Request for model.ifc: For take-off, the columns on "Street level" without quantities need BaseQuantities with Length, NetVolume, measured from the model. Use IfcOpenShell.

First a look at what the model holds.

```python
import ifcopenshell
import ifcopenshell.util.element
import ifcopenshell.util.unit

model = ifcopenshell.open("model.ifc")
print(model.schema)
for unit_type in ("LENGTHUNIT", "AREAUNIT", "VOLUMEUNIT"):
    print(unit_type, ifcopenshell.util.unit.calculate_unit_scale(model, unit_type))
storey = next(s for s in model.by_type("IfcBuildingStorey") if s.Name == "Street level")
columns = [e for e in ifcopenshell.util.element.get_decomposition(storey) if e.is_a("IfcColumn")]
for e in sorted(columns, key=lambda e: e.id()):
    print(e.id(), e.is_a(), e.Name, list(ifcopenshell.util.element.get_psets(e, qtos_only=True)), sep=" | ")
```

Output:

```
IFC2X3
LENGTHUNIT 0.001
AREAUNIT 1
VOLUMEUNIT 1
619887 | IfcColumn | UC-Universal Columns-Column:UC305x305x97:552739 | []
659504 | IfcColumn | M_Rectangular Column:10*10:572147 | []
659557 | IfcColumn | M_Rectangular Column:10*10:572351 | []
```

```python
import ifcopenshell
import ifcopenshell.api.pset
import ifcopenshell.geom
import ifcopenshell.util.element
import ifcopenshell.util.shape
import ifcopenshell.util.unit

model = ifcopenshell.open("model.ifc")
unit_scale = ifcopenshell.util.unit.calculate_unit_scale(model)
volume_scale = ifcopenshell.util.unit.calculate_unit_scale(model, "VOLUMEUNIT")
settings = ifcopenshell.geom.settings()

storey = next(s for s in model.by_type("IfcBuildingStorey") if s.Name == "Street level")
columns = [e for e in ifcopenshell.util.element.get_decomposition(storey) if e.is_a("IfcColumn")]

for e in sorted(columns, key=lambda e: e.id()):
    if ifcopenshell.util.element.get_psets(e, qtos_only=True, should_inherit=False):
        continue
    # Geometry comes back in metres, in the element's own axes.
    shape = ifcopenshell.geom.create_shape(settings, e)
    values = {
        "Length": ifcopenshell.util.shape.get_z(shape.geometry) / unit_scale,
        "NetVolume": ifcopenshell.util.shape.get_volume(shape.geometry) / volume_scale,
    }
    qto = ifcopenshell.api.pset.add_qto(model, product=e, name="BaseQuantities")
    ifcopenshell.api.pset.edit_qto(model, qto=qto, properties=values)
    print(e.id(), {k: round(v, 3) for k, v in values.items()})

model.write("model_rev.ifc")
```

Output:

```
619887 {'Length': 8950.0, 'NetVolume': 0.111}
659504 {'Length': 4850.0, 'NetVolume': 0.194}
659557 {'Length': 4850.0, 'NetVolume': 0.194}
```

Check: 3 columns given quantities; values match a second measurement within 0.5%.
